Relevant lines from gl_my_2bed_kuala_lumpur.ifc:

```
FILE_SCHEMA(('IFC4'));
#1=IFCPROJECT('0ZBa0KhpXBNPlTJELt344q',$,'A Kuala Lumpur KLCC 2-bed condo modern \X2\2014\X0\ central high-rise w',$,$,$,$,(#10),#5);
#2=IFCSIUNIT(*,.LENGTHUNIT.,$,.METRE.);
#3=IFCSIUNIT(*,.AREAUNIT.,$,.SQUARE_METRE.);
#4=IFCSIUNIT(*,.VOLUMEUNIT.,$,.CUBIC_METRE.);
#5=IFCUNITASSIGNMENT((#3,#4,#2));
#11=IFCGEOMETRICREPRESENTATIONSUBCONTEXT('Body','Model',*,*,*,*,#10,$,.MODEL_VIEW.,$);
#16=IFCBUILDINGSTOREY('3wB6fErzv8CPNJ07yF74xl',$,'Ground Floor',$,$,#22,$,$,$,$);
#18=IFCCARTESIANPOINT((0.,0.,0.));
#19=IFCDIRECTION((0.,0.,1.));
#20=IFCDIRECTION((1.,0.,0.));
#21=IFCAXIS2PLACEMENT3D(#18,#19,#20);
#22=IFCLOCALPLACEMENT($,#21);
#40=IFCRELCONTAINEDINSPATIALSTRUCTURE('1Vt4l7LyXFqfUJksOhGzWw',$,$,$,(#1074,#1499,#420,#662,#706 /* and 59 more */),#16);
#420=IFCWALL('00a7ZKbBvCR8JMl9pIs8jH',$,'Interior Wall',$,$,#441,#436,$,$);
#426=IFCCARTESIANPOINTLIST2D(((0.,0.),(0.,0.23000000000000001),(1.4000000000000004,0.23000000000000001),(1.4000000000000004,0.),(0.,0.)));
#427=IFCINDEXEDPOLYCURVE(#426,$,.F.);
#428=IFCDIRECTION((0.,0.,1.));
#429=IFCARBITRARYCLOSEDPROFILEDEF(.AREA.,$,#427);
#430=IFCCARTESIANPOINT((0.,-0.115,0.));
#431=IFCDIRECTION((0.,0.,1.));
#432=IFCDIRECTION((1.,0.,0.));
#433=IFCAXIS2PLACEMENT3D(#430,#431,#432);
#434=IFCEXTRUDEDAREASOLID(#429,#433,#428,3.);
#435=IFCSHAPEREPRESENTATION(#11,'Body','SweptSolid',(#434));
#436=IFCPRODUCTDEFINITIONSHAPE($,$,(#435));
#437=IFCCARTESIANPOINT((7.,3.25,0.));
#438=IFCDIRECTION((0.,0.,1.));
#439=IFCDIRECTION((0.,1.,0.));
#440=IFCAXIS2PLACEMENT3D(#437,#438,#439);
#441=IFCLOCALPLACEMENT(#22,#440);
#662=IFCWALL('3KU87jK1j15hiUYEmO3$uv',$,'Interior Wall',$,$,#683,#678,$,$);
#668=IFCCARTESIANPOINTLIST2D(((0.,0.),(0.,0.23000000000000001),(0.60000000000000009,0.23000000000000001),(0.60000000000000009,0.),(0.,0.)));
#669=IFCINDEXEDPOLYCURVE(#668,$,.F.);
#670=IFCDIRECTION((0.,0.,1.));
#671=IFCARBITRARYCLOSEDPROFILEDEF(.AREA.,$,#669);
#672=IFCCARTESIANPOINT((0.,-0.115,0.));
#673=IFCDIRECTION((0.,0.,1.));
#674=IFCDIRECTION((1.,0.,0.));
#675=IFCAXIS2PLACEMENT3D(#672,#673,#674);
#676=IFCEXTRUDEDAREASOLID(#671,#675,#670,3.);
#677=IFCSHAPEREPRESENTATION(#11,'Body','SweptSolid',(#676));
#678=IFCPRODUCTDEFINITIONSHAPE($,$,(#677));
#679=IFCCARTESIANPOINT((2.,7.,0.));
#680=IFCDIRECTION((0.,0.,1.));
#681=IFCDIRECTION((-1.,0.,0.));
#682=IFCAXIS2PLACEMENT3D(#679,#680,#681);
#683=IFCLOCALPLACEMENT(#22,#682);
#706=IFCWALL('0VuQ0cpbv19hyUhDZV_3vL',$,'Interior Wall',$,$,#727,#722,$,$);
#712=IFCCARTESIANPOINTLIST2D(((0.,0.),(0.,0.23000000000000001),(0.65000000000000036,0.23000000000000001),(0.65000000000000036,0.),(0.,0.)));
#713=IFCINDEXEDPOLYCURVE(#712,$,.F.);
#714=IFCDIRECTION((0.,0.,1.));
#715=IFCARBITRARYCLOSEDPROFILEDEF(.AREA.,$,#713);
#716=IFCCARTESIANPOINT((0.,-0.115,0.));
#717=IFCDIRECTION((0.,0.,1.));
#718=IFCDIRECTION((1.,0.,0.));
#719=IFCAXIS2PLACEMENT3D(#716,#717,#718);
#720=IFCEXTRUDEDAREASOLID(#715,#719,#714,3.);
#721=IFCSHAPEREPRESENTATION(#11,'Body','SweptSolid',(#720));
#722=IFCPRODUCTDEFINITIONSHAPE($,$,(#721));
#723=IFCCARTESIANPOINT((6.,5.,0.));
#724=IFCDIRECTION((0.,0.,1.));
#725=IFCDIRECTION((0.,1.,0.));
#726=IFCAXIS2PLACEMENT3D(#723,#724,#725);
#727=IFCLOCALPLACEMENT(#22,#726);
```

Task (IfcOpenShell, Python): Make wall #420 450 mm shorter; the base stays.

```python
import ifcopenshell
import ifcopenshell.geom
import ifcopenshell.util.representation
import ifcopenshell.util.shape

model = ifcopenshell.open("gl_my_2bed_kuala_lumpur.ifc")
settings = ifcopenshell.geom.settings()


def volume(element):
    """Net volume in cubic metres, openings subtracted."""
    shape = ifcopenshell.geom.create_shape(settings, element)
    return ifcopenshell.util.shape.get_volume(shape.geometry)


wall = model.by_guid("00a7ZKbBvCR8JMl9pIs8jH")
before = volume(wall)

body = ifcopenshell.util.representation.get_representation(wall, "Model", "Body")
solid = body.Items[0]
old_height = solid.Depth
solid.Depth -= 0.45
after = volume(wall)

print(f"height {old_height:g} -> {solid.Depth:g}, volume {before:.3f} -> {after:.3f} m3")

model.write("gl_my_2bed_kuala_lumpur-out.ifc")
```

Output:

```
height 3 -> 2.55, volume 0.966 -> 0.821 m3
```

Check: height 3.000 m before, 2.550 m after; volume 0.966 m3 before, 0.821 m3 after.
